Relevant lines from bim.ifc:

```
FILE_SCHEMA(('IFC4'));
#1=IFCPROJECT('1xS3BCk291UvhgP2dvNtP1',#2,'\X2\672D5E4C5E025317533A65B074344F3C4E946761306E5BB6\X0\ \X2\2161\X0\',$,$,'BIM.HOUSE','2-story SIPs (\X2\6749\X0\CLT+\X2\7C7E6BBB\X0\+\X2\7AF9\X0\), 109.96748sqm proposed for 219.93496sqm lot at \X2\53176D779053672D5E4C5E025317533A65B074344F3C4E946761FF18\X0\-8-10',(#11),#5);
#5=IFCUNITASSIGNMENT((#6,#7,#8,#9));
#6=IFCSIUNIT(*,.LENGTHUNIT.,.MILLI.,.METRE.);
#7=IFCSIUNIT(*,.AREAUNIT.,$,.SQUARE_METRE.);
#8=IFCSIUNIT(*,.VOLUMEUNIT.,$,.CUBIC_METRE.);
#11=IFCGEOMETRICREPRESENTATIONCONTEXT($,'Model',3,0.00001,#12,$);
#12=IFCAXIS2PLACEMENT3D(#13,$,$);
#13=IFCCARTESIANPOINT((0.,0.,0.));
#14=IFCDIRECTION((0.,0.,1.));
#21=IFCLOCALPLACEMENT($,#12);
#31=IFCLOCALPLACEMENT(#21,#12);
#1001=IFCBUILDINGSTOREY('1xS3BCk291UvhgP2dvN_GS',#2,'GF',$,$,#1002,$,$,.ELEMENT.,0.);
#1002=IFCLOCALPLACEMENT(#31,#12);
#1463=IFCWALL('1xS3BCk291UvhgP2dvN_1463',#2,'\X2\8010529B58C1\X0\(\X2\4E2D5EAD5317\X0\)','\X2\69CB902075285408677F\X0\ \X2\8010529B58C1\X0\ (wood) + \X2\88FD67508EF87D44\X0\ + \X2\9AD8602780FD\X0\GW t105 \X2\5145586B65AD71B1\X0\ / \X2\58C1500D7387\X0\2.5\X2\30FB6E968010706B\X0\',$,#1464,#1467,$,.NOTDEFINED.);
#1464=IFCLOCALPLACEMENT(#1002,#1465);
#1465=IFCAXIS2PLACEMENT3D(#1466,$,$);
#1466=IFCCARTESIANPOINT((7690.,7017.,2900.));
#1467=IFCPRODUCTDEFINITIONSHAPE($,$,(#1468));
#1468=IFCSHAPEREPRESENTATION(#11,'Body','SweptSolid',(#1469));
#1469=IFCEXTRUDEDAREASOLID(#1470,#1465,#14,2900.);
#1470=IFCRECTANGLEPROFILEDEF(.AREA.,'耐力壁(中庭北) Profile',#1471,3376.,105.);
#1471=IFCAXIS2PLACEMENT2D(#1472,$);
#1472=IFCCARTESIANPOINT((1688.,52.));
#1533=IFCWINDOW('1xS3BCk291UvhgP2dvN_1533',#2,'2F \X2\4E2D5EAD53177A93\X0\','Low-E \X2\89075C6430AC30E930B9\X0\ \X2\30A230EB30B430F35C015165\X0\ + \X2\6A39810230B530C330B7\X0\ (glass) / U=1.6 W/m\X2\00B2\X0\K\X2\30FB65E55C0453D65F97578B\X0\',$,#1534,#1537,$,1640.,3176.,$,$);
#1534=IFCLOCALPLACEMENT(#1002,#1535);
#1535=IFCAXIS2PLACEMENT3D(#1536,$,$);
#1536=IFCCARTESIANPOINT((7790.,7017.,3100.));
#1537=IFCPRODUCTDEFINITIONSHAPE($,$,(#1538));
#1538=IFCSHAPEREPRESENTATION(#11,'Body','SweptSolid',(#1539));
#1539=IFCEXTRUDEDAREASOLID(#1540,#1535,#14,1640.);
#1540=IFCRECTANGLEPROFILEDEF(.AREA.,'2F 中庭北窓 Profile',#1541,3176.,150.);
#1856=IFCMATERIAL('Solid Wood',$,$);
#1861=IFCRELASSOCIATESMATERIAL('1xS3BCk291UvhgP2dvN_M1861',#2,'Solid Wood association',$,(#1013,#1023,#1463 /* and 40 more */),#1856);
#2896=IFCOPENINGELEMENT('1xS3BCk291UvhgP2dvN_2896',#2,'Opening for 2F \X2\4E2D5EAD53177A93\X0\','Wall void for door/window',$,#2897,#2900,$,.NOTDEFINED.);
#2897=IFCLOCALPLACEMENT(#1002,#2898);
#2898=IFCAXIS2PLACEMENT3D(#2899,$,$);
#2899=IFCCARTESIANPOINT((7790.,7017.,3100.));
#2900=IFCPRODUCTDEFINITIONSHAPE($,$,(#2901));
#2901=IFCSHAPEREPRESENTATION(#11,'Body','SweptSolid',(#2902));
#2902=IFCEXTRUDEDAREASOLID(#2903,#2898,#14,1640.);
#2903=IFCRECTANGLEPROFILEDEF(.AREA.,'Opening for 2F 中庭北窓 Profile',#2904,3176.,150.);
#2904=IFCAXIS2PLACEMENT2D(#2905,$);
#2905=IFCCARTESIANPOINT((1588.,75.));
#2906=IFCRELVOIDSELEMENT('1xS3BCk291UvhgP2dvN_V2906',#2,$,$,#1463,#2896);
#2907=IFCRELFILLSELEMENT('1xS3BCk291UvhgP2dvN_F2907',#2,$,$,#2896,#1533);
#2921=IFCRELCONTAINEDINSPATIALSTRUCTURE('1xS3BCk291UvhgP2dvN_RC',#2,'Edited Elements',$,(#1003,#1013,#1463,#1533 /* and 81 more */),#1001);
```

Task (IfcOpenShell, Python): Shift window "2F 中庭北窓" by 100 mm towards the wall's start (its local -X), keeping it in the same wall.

```python
import ifcopenshell
import ifcopenshell.api.geometry
import ifcopenshell.util.placement
import ifcopenshell.util.unit

model = ifcopenshell.open("bim.ifc")
unit_scale = ifcopenshell.util.unit.calculate_unit_scale(model)

window = model.by_guid("1xS3BCk291UvhgP2dvN_1533")
opening = window.FillsVoids[0].RelatingOpeningElement
wall = opening.VoidsElements[0].RelatingBuildingElement

wall_matrix = ifcopenshell.util.placement.get_local_placement(wall.ObjectPlacement)
shift = wall_matrix[:3, 0] * -0.1 / unit_scale
before = ifcopenshell.util.placement.get_local_placement(window.ObjectPlacement)[:3, 3].copy()

# The window is not placed relative to its opening, so move both.
for product in (opening, window):
    matrix = ifcopenshell.util.placement.get_local_placement(product.ObjectPlacement)
    matrix[:3, 3] += shift
    ifcopenshell.api.geometry.edit_object_placement(model, product=product, matrix=matrix, is_si=False)

after = ifcopenshell.util.placement.get_local_placement(window.ObjectPlacement)[:3, 3]
print("window moved by", (after - before).round(3) + 0.0)

model.write("bim_rev.ifc")
```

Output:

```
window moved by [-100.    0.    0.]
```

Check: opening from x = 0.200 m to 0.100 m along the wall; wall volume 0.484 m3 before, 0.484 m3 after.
